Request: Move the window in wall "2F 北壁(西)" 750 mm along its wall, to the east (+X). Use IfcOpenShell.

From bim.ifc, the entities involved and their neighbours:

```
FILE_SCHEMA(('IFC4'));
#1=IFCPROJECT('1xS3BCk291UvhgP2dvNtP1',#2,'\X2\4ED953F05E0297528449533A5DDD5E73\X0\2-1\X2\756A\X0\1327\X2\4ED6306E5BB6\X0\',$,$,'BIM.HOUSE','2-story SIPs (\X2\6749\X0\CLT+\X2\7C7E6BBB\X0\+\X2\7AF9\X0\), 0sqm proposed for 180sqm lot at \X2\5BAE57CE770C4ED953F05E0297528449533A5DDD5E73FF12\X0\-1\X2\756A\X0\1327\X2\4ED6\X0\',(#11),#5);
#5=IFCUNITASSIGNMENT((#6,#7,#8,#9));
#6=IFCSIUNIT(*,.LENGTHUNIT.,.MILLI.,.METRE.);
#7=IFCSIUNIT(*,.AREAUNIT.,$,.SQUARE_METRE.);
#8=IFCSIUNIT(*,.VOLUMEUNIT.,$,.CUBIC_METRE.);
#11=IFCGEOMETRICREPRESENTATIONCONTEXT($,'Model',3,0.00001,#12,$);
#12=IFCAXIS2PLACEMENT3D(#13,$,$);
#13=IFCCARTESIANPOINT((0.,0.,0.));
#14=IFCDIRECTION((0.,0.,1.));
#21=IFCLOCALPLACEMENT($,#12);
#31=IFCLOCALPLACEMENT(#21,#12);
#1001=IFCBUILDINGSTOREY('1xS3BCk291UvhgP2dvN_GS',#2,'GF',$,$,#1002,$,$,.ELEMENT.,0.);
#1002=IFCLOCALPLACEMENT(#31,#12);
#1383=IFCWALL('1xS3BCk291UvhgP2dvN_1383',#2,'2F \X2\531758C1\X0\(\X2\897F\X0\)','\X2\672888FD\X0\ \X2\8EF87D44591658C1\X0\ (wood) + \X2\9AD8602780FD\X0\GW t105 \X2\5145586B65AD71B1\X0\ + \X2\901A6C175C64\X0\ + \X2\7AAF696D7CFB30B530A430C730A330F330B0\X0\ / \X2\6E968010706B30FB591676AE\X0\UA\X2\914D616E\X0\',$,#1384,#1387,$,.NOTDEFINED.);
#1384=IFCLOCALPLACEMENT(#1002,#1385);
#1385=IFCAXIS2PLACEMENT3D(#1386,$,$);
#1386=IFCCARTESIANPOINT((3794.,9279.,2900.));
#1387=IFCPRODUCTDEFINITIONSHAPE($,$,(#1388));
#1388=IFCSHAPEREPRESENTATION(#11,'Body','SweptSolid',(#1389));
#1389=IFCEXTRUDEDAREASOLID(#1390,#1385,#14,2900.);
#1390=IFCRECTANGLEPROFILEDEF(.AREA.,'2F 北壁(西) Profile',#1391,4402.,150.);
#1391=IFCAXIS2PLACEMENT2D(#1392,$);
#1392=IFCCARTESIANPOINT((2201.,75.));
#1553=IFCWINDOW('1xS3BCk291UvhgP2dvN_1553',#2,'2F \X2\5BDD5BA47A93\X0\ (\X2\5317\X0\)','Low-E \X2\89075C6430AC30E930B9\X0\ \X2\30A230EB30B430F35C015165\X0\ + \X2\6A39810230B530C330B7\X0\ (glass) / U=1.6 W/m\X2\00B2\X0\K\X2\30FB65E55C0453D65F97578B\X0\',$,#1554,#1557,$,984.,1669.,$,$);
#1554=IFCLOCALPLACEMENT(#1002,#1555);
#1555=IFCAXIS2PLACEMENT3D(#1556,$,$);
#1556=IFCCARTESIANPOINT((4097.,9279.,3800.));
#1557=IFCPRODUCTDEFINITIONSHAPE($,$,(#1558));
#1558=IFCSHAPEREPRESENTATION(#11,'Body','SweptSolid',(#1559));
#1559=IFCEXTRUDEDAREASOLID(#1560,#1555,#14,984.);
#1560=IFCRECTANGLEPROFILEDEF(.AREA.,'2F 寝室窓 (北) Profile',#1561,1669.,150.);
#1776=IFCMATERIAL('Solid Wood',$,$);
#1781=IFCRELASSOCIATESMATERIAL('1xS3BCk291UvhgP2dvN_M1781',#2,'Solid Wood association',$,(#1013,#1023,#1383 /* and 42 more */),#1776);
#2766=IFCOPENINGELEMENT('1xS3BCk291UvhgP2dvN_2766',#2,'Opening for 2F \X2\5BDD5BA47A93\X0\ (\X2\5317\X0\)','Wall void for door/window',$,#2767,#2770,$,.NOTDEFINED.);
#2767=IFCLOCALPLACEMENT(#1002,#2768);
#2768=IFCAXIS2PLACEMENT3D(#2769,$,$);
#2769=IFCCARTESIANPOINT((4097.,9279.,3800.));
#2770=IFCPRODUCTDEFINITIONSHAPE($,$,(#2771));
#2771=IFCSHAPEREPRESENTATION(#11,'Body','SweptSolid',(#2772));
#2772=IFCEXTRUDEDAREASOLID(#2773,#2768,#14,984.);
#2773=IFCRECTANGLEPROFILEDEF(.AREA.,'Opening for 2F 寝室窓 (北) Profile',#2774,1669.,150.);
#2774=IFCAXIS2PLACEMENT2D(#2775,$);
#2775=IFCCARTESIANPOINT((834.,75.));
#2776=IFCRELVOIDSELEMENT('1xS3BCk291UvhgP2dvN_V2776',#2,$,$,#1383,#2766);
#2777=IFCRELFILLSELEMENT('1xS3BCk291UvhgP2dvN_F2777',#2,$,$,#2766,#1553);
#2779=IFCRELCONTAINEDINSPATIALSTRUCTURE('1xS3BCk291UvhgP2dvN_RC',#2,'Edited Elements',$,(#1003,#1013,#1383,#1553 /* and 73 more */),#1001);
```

```python
import ifcopenshell
import ifcopenshell.api.geometry
import ifcopenshell.util.placement

model = ifcopenshell.open("bim.ifc")

window = model.by_guid("1xS3BCk291UvhgP2dvN_1553")
opening = window.FillsVoids[0].RelatingOpeningElement
wall = opening.VoidsElements[0].RelatingBuildingElement

wall_matrix = ifcopenshell.util.placement.get_local_placement(wall.ObjectPlacement)
shift = wall_matrix[:3, 0] * 750.0
before = ifcopenshell.util.placement.get_local_placement(window.ObjectPlacement)[:3, 3].copy()

# The window is not placed relative to its opening, so move both.
for product in (opening, window):
    matrix = ifcopenshell.util.placement.get_local_placement(product.ObjectPlacement)
    matrix[:3, 3] += shift
    ifcopenshell.api.geometry.edit_object_placement(model, product=product, matrix=matrix, is_si=False)

after = ifcopenshell.util.placement.get_local_placement(window.ObjectPlacement)[:3, 3]
print("window moved by", (after - before).round(3) + 0.0)

model.write("bim_edited.ifc")
```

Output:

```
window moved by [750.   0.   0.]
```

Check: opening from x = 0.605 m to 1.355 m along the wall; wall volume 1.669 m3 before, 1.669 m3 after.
